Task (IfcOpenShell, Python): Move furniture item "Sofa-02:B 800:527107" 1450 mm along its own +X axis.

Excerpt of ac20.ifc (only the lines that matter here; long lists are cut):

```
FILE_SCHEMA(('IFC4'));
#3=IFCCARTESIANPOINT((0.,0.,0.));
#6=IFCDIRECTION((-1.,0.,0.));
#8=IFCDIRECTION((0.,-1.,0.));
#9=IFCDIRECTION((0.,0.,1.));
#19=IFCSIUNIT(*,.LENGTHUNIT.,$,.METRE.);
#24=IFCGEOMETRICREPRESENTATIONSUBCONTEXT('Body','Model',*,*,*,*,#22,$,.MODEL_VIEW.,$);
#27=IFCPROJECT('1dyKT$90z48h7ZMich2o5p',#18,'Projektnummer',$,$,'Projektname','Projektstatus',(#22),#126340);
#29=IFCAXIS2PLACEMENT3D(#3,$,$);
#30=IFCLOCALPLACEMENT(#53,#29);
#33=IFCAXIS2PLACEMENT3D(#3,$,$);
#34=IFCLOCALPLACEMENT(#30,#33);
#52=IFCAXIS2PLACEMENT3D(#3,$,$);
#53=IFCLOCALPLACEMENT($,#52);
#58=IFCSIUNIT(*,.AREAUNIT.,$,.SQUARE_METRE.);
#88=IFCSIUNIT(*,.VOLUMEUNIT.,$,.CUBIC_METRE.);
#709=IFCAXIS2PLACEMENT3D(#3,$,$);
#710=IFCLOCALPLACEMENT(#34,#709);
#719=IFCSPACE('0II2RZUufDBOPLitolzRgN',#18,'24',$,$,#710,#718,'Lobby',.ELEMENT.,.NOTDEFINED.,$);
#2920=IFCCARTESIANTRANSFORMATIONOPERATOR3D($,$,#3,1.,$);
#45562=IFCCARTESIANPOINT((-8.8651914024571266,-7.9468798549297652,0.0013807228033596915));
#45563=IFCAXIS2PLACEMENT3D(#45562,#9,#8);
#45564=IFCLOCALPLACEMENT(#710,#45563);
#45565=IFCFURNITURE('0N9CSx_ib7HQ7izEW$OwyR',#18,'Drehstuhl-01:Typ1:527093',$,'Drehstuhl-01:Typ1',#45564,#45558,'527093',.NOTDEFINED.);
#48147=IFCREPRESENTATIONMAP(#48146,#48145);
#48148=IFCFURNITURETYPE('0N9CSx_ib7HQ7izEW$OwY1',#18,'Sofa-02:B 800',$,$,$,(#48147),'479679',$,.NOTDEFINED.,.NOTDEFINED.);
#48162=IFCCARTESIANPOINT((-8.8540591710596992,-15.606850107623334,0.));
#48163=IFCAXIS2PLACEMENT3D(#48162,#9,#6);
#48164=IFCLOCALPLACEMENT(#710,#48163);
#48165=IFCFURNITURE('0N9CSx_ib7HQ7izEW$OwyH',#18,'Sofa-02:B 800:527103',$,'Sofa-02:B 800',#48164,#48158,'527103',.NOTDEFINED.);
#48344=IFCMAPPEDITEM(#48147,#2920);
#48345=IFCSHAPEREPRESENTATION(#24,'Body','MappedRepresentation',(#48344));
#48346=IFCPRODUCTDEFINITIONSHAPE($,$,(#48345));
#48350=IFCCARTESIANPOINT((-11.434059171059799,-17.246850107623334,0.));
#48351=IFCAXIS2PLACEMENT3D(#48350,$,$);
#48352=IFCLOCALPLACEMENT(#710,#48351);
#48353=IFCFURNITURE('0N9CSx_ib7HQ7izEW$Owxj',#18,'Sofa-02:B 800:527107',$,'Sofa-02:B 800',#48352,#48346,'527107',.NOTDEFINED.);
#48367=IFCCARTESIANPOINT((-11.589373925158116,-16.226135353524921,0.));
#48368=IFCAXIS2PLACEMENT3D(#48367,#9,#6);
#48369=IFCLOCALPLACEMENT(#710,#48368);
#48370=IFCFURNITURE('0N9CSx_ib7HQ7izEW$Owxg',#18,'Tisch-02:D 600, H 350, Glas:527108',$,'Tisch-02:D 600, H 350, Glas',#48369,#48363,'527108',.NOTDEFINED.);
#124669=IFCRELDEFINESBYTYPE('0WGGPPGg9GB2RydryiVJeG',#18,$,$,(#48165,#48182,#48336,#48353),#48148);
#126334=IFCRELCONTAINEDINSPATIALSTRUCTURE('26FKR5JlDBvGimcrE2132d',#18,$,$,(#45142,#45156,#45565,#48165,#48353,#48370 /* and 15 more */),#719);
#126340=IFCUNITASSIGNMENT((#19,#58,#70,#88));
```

```python
import ifcopenshell
import ifcopenshell.api.geometry
import ifcopenshell.util.placement
import ifcopenshell.util.unit

model = ifcopenshell.open("ac20.ifc")
unit_scale = ifcopenshell.util.unit.calculate_unit_scale(model)

item = model.by_guid("0N9CSx_ib7HQ7izEW$Owxj")
matrix = ifcopenshell.util.placement.get_local_placement(item.ObjectPlacement)
matrix[:3, 3] += matrix[:3, 0] * 1.45 / unit_scale
ifcopenshell.api.geometry.edit_object_placement(model, product=item, matrix=matrix, is_si=False)

print(ifcopenshell.util.placement.get_local_placement(item.ObjectPlacement).round(3) + 0.0)

model.write("ac20_rev.ifc")
```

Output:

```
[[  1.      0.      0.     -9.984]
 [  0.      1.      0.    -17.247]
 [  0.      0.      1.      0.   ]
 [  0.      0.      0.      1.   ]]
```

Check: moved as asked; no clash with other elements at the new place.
